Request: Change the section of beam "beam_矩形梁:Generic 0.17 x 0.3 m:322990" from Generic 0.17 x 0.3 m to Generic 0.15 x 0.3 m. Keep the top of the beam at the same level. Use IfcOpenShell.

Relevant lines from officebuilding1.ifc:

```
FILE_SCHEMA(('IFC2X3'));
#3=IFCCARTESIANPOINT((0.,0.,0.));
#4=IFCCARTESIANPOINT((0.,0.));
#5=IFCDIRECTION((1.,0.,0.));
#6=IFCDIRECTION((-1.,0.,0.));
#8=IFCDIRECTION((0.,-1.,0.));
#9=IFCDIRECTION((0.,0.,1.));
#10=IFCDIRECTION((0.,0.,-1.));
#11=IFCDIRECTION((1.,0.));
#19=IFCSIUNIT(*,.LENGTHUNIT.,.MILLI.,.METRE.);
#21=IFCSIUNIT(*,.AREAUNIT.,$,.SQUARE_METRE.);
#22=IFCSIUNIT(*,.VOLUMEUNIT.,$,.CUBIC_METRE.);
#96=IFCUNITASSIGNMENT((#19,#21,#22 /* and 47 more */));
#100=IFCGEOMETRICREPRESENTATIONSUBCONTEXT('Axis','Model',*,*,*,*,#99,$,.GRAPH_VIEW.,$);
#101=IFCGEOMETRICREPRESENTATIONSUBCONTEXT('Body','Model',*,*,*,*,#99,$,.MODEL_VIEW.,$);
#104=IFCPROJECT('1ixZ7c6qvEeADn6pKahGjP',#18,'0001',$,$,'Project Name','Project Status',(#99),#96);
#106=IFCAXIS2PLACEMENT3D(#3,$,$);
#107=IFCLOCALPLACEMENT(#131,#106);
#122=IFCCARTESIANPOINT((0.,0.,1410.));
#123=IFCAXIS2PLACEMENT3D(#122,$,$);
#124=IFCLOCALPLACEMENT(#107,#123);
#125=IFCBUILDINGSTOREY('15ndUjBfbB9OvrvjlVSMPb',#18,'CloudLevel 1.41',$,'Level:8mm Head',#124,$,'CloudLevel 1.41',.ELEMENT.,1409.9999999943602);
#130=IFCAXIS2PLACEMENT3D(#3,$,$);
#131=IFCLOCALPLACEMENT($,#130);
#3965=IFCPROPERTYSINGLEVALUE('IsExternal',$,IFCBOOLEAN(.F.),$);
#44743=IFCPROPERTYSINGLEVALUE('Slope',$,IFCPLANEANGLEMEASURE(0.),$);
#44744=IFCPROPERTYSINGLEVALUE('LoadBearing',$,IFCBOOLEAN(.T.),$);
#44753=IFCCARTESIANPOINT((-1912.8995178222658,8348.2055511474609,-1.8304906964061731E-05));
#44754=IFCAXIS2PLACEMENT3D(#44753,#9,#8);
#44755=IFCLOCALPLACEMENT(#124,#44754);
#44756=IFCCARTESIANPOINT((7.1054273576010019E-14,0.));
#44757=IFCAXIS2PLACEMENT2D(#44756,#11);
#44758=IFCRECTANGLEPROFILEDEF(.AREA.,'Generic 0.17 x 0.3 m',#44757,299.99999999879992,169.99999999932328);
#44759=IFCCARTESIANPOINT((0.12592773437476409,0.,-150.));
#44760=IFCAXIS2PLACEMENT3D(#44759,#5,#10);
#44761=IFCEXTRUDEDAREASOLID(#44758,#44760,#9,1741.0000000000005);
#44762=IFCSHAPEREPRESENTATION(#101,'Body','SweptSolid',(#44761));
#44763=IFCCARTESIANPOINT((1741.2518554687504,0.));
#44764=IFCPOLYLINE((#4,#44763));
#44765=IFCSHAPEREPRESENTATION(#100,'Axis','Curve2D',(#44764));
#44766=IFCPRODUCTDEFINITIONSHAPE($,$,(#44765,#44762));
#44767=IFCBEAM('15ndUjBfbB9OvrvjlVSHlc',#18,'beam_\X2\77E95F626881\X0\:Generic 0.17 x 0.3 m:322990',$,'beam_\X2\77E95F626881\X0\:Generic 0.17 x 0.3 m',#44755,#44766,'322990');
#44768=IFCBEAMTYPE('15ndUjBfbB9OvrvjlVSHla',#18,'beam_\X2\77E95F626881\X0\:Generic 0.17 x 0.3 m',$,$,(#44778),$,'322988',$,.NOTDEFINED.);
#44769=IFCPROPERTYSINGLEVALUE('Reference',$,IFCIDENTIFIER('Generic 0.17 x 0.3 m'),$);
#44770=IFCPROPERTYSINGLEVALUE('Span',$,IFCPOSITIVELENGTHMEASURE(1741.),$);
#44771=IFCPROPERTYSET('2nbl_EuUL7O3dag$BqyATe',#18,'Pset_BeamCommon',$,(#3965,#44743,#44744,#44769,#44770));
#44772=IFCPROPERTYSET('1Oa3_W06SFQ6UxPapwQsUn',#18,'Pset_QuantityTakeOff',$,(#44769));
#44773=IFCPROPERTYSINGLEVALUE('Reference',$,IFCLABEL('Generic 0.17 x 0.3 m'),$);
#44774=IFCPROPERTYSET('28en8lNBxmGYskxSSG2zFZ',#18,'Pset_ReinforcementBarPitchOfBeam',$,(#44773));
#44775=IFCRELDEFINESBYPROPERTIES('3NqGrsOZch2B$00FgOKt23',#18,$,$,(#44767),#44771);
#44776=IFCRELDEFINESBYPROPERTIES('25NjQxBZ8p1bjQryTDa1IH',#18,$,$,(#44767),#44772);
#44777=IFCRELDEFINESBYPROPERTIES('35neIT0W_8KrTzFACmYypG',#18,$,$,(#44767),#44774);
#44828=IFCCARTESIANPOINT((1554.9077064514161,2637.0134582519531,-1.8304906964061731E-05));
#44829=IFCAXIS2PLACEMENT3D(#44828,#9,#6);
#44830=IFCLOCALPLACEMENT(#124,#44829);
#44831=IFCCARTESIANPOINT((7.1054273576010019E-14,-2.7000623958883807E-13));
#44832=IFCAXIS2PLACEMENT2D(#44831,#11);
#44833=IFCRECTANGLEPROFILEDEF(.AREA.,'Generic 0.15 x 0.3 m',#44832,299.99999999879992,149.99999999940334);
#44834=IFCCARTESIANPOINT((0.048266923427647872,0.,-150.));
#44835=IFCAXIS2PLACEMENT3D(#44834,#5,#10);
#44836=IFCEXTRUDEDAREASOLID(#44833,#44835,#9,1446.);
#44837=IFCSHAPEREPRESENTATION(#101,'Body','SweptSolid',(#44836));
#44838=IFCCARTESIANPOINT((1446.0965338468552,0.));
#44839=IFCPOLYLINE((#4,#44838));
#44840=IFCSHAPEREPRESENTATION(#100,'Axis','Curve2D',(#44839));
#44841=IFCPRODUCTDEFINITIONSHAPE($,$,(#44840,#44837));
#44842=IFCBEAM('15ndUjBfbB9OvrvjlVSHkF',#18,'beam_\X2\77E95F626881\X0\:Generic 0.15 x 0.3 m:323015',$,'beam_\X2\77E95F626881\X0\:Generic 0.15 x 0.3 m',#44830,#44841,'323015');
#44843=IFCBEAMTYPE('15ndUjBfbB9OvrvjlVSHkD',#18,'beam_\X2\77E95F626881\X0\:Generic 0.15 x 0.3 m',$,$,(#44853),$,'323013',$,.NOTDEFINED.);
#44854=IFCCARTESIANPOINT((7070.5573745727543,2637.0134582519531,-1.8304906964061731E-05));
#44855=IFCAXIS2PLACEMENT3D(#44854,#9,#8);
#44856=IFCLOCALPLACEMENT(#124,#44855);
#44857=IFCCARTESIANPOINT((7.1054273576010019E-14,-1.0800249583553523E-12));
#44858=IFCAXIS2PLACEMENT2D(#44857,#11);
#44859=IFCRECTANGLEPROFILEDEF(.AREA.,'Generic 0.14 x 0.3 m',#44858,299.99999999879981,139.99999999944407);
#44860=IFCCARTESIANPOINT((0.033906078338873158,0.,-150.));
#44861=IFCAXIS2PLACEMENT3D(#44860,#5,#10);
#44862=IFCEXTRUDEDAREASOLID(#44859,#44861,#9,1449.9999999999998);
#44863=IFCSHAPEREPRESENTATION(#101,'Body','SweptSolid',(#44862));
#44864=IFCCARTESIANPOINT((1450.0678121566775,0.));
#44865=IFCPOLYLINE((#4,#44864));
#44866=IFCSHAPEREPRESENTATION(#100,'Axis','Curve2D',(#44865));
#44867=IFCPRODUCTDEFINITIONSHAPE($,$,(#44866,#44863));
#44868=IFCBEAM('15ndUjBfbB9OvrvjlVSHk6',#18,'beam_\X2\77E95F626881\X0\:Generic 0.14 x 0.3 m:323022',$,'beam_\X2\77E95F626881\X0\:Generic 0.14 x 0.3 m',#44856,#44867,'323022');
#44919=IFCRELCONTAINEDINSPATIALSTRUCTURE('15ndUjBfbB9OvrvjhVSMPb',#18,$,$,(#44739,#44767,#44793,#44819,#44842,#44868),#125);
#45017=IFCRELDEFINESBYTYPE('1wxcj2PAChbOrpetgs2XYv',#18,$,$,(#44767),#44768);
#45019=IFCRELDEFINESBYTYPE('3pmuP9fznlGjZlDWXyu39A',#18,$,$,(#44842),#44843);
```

```python
import ifcopenshell
import ifcopenshell.api.pset
import ifcopenshell.api.type
import ifcopenshell.util.element
import ifcopenshell.util.representation

model = ifcopenshell.open("officebuilding1.ifc")

member = model.by_guid("15ndUjBfbB9OvrvjlVSHlc")
source = next(p for p in model.by_type("IfcRectangleProfileDef") if p.ProfileName == "Generic 0.15 x 0.3 m")

body = ifcopenshell.util.representation.get_representation(member, "Model", "Body")
solid = body.Items[0]
old_profile = solid.SweptArea

# Copy the section's sizes but keep this member's own profile position.
profile = ifcopenshell.util.element.copy(model, source)
# Profiles are centred, so shift by half the change in depth to hold the top.
shift = (old_profile.XDim - profile.XDim) / 2
x, y = old_profile.Position.Location.Coordinates
up = (-1.0, 0.0)  # upwards, in the solid's own plane
location = model.createIfcCartesianPoint((x + up[0] * shift, y + up[1] * shift))
profile.Position = model.createIfcAxis2Placement2D(location, old_profile.Position.RefDirection)
solid.SweptArea = profile
if not model.get_total_inverses(old_profile):
    ifcopenshell.util.element.remove_deep2(model, old_profile)

new_type = model.by_id(44843)
ifcopenshell.api.type.assign_type(
    model, related_objects=[member], relating_type=new_type, should_map_representations=False
)
member.Name = member.Name.replace("Generic 0.17 x 0.3 m", "Generic 0.15 x 0.3 m")
member.ObjectType = "beam_矩形梁:Generic 0.15 x 0.3 m"
pset = model.by_id(ifcopenshell.util.element.get_pset(member, "Pset_BeamCommon", should_inherit=False)["id"])
ifcopenshell.api.pset.edit_pset(model, pset=pset, properties={"Reference": "Generic 0.15 x 0.3 m"})
pset = model.by_id(ifcopenshell.util.element.get_pset(member, "Pset_QuantityTakeOff", should_inherit=False)["id"])
ifcopenshell.api.pset.edit_pset(model, pset=pset, properties={"Reference": "Generic 0.15 x 0.3 m"})
pset = model.by_id(ifcopenshell.util.element.get_pset(member, "Pset_ReinforcementBarPitchOfBeam", should_inherit=False)["id"])
ifcopenshell.api.pset.edit_pset(model, pset=pset, properties={"Reference": "Generic 0.15 x 0.3 m"})

print(solid.SweptArea)

model.write("officebuilding1_updated.ifc")
```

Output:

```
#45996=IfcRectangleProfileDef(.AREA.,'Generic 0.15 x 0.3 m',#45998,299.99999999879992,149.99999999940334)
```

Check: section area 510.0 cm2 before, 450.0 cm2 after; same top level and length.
